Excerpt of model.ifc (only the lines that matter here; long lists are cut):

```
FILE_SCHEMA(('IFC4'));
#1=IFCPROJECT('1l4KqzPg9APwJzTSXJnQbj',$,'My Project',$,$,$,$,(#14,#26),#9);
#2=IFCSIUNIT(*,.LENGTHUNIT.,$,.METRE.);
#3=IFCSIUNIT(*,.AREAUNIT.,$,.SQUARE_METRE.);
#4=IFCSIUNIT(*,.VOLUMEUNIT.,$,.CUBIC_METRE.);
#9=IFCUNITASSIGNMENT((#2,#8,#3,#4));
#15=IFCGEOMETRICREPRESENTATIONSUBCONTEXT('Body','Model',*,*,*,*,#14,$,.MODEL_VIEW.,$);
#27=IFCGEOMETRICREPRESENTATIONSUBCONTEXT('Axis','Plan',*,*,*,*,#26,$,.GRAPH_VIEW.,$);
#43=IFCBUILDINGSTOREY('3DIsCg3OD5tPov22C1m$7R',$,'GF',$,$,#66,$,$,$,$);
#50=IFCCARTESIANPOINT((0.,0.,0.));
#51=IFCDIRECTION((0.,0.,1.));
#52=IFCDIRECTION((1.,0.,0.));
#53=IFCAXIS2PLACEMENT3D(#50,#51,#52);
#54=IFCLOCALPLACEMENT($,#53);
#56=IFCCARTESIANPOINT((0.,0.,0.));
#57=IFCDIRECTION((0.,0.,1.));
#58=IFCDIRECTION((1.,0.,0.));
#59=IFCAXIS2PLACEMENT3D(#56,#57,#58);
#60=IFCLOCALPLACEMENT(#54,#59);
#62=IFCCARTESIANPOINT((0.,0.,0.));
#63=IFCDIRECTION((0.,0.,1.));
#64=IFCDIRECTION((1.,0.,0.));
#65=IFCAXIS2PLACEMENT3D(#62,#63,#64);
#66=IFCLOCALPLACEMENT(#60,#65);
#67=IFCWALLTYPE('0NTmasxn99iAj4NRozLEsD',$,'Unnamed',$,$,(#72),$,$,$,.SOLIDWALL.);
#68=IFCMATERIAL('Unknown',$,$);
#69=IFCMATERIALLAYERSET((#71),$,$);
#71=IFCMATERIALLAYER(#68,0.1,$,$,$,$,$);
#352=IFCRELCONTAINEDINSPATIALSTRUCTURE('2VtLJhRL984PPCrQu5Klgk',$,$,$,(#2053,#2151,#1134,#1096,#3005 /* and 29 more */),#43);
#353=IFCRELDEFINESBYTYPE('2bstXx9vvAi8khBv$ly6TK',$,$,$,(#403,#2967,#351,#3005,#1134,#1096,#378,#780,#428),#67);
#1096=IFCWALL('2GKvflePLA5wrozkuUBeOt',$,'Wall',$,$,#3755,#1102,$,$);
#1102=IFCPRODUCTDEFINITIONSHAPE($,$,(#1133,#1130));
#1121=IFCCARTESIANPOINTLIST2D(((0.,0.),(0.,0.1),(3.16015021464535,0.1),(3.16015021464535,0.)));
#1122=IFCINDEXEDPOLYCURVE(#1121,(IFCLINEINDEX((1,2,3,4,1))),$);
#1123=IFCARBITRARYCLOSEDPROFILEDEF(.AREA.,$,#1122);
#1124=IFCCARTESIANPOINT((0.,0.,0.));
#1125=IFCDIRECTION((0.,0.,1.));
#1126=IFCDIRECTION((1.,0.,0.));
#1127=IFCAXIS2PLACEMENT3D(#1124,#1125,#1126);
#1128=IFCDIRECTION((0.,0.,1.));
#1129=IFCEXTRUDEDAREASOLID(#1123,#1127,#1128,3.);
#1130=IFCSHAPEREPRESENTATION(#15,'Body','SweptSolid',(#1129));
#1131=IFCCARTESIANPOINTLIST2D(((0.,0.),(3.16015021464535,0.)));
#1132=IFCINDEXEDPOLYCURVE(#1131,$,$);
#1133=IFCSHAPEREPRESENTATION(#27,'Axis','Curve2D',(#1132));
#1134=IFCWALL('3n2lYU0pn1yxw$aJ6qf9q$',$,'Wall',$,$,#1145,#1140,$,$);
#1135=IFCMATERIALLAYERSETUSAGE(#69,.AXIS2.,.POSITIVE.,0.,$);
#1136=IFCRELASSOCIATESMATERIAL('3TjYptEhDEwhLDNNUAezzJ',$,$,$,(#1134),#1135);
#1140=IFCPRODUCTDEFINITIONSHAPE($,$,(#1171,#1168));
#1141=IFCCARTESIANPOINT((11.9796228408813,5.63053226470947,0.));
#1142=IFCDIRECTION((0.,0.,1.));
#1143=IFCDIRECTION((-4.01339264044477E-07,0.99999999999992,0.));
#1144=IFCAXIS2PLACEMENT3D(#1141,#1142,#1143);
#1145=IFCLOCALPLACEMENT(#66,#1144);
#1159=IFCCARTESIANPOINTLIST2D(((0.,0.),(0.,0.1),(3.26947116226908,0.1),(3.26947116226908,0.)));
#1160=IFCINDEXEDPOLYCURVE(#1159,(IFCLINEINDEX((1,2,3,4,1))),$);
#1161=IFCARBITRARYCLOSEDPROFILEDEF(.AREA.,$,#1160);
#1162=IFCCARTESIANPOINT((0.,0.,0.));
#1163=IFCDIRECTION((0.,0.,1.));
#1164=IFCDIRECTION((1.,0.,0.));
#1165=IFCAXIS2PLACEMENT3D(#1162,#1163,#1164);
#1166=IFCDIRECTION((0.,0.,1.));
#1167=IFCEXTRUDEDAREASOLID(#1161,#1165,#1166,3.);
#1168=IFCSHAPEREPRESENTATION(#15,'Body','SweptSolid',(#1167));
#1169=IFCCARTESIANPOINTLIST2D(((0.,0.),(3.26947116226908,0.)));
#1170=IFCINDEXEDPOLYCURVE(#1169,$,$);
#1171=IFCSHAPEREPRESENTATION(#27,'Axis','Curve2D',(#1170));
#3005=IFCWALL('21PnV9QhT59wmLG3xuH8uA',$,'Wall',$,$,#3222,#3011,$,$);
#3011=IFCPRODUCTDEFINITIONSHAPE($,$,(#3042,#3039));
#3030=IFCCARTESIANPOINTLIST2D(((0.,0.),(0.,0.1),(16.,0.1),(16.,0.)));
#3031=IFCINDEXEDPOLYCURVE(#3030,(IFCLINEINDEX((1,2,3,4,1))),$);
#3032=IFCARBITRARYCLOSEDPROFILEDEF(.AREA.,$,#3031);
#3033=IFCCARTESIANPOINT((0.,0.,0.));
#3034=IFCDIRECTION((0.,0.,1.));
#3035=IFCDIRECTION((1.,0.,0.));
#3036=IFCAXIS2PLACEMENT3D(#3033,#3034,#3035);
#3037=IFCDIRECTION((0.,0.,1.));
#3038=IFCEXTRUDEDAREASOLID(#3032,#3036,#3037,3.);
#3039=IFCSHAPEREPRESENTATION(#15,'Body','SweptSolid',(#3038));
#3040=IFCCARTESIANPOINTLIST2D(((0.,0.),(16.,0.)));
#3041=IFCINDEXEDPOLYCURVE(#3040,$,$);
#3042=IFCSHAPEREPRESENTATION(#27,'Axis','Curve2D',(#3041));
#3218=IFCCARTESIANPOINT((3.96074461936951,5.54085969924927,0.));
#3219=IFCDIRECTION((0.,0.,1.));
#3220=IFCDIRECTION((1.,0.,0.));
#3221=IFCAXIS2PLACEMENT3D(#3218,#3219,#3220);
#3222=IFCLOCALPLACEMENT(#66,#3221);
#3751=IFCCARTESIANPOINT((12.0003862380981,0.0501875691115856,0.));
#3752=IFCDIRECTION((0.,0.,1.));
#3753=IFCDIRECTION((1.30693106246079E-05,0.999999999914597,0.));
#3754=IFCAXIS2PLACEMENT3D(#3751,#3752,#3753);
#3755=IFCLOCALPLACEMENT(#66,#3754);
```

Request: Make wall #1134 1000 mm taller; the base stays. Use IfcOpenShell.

```python
import ifcopenshell
import ifcopenshell.geom
import ifcopenshell.util.representation
import ifcopenshell.util.shape
import ifcopenshell.util.unit

model = ifcopenshell.open("model.ifc")
unit_scale = ifcopenshell.util.unit.calculate_unit_scale(model)
settings = ifcopenshell.geom.settings()


def volume(element):
    """Net volume in cubic metres, openings subtracted."""
    shape = ifcopenshell.geom.create_shape(settings, element)
    return ifcopenshell.util.shape.get_volume(shape.geometry)


wall = model.by_guid("3n2lYU0pn1yxw$aJ6qf9q$")
before = volume(wall)

body = ifcopenshell.util.representation.get_representation(wall, "Model", "Body")
solid = body.Items[0]
old_height = solid.Depth
solid.Depth += 1 / unit_scale
after = volume(wall)

print(f"height {old_height:g} -> {solid.Depth:g}, volume {before:.3f} -> {after:.3f} m3")

model.write("model_updated.ifc")
```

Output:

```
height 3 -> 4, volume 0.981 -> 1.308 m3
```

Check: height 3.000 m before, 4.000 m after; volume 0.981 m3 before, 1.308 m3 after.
